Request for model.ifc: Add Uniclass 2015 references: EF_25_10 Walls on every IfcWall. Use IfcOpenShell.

First a look at what the model holds.

```python
import ifcopenshell

model = ifcopenshell.open("model.ifc")
print(model.schema)
print("classifications:", [c.Name for c in model.by_type("IfcClassification")])
for ifc_class in ("IfcDoor", "IfcRoof", "IfcStair", "IfcWall", "IfcWindow"):
    print(ifc_class, len(model.by_type(ifc_class)))
```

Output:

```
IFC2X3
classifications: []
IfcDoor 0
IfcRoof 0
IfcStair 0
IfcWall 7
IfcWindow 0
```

```python
import ifcopenshell
import ifcopenshell.api.classification

model = ifcopenshell.open("model.ifc")

# IFC2X3 requires Source and Edition and has no link from the project to the system.
system = model.create_entity("IfcClassification", Source="NBS", Edition="2015", Name="Uniclass 2015")

codes = {
    "IfcWall": ("EF_25_10", "Walls"),
}
for ifc_class, (code, name) in codes.items():
    products = model.by_type(ifc_class)
    ifcopenshell.api.classification.add_reference(
        model, products=products, classification=system, identification=code, name=name
    )
    print(code, len(products))

model.write("model_edited.ifc")
```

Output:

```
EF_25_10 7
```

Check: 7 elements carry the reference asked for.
